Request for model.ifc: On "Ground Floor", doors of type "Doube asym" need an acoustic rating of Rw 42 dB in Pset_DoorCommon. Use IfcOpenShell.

First a look at what the model holds.

```python
import ifcopenshell
import ifcopenshell.util.element

model = ifcopenshell.open("model.ifc")
print(model.schema)
storey = next(s for s in model.by_type("IfcBuildingStorey") if s.Name == "Ground Floor")
doors = [e for e in ifcopenshell.util.element.get_decomposition(storey) if e.is_a("IfcDoor")]
seen = {}
for e in doors:
    element_type = ifcopenshell.util.element.get_type(e)
    key = (element_type.Name if element_type != e and element_type else None, ifcopenshell.util.element.get_pset(e, "Pset_DoorCommon", "AcousticRating"))
    seen[key] = seen.get(key, 0) + 1
for (name, value), count in sorted(seen.items(), key=str):
    print(count, "x", name, "|", value)
```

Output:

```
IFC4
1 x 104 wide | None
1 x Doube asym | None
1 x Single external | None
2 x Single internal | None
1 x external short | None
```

```python
import ifcopenshell
import ifcopenshell.api.pset
import ifcopenshell.util.element

model = ifcopenshell.open("model.ifc")

storey = next(s for s in model.by_type("IfcBuildingStorey") if s.Name == "Ground Floor")
doors = [e for e in ifcopenshell.util.element.get_decomposition(storey) if e.is_a("IfcDoor")]

count = 0
for e in doors:
    element_type = ifcopenshell.util.element.get_type(e)
    if element_type in (None, e) or element_type.Name != "Doube asym":
        continue
    # add_pset returns the element's existing set when there is one.
    pset = ifcopenshell.api.pset.add_pset(model, product=e, name="Pset_DoorCommon")
    ifcopenshell.api.pset.edit_pset(model, pset=pset, properties={"AcousticRating": "Rw 42 dB"})
    count += 1

print(count, "doors updated")

model.write("model-out.ifc")
```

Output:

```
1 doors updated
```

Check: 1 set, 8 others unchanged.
